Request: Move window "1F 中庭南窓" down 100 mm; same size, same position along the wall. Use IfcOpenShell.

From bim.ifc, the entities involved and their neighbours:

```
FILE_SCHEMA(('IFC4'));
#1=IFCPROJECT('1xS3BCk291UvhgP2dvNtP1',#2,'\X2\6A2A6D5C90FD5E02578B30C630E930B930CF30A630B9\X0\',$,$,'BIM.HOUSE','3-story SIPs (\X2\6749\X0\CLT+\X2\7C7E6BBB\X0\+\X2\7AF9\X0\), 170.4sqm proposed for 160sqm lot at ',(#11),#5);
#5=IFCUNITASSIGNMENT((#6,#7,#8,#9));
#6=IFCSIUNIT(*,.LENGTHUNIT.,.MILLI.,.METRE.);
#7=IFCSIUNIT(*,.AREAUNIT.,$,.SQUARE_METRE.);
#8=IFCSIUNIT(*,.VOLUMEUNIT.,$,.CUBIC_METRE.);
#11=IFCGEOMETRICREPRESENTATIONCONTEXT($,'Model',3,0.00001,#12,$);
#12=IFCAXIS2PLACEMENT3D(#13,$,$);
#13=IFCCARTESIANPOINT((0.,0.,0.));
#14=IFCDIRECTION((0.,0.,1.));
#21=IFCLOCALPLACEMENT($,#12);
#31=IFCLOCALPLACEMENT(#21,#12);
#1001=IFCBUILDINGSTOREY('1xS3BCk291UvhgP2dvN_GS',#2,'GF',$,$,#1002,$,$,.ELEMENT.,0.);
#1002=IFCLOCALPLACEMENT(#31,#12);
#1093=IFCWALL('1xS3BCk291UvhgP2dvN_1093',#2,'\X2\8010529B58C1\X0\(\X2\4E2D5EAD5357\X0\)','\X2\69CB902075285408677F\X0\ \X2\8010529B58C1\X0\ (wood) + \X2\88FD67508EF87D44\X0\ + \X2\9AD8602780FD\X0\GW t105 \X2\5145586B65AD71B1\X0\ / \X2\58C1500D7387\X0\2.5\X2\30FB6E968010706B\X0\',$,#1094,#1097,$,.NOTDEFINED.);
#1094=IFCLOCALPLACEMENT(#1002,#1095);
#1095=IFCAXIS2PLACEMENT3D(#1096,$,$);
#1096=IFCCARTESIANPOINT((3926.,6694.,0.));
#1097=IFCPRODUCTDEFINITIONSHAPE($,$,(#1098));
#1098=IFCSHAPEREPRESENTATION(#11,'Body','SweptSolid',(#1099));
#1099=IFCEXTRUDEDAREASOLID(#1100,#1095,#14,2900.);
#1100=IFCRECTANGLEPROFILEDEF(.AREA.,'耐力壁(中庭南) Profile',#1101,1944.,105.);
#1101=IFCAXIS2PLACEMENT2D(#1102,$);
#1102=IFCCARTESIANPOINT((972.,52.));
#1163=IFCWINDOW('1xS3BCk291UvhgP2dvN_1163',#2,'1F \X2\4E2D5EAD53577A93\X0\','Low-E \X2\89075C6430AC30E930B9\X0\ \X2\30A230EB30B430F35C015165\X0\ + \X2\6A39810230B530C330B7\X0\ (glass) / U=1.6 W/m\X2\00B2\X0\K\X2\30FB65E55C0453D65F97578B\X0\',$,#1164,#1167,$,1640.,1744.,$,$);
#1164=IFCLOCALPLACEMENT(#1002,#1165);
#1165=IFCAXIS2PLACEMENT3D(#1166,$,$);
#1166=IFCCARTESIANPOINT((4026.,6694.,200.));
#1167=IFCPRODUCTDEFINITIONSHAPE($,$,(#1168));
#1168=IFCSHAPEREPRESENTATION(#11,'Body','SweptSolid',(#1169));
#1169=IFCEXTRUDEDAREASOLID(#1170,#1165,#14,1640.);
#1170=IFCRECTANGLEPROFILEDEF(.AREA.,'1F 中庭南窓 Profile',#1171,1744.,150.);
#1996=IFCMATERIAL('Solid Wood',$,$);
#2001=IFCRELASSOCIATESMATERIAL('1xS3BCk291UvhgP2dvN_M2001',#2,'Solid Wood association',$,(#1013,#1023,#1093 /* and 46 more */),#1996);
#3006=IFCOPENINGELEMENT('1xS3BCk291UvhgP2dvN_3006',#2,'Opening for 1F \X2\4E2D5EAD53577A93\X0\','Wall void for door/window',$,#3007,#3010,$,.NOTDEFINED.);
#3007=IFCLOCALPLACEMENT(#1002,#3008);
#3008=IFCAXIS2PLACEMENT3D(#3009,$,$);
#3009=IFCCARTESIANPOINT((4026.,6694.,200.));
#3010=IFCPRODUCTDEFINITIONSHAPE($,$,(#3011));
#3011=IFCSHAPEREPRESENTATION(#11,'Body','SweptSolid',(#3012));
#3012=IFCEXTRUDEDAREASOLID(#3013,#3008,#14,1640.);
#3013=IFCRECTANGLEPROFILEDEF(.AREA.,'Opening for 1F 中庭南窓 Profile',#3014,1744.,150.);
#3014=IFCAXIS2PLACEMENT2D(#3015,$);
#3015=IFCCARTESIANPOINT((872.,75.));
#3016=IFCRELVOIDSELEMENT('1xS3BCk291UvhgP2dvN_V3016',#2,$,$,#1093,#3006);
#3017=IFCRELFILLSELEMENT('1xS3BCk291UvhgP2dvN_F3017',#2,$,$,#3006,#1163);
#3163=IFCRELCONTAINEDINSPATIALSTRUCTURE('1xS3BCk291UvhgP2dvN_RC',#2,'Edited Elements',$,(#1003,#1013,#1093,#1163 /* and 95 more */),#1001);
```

```python
import numpy as np
import ifcopenshell
import ifcopenshell.api.geometry
import ifcopenshell.util.placement
import ifcopenshell.util.unit

model = ifcopenshell.open("bim.ifc")
unit_scale = ifcopenshell.util.unit.calculate_unit_scale(model)

window = model.by_guid("1xS3BCk291UvhgP2dvN_1163")
opening = window.FillsVoids[0].RelatingOpeningElement
dz = -100.0

shift = np.array([0.0, 0.0, dz])
# The window is not placed relative to its opening, so move both.
for product in (opening, window):
    matrix = ifcopenshell.util.placement.get_local_placement(product.ObjectPlacement)
    matrix[:3, 3] += shift
    ifcopenshell.api.geometry.edit_object_placement(model, product=product, matrix=matrix, is_si=False)

print(f"moved by {dz * unit_scale:+.3f} m")

model.write("bim_updated.ifc")
```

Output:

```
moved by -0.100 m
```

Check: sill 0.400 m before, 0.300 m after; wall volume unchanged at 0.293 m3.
